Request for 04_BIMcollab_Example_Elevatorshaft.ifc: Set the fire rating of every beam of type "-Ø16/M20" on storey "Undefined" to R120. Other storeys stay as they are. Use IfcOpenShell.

First a look at what the model holds.

```python
import ifcopenshell
import ifcopenshell.util.element

model = ifcopenshell.open("04_BIMcollab_Example_Elevatorshaft.ifc")
print(model.schema)
storey = next(s for s in model.by_type("IfcBuildingStorey") if s.Name == "Undefined")
beams = [e for e in ifcopenshell.util.element.get_decomposition(storey) if e.is_a("IfcBeam")]
seen = {}
for e in beams:
    element_type = ifcopenshell.util.element.get_type(e)
    key = (element_type.Name if element_type != e and element_type else None, ifcopenshell.util.element.get_pset(e, "Pset_BeamCommon", "FireRating"))
    seen[key] = seen.get(key, 0) + 1
for (name, value), count in sorted(seen.items(), key=str):
    print(count, "x", name, "|", value)
```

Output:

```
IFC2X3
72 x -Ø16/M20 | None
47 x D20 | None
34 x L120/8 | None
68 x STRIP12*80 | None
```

```python
import ifcopenshell
import ifcopenshell.api.pset
import ifcopenshell.util.element

model = ifcopenshell.open("04_BIMcollab_Example_Elevatorshaft.ifc")

storey = next(s for s in model.by_type("IfcBuildingStorey") if s.Name == "Undefined")
beams = [e for e in ifcopenshell.util.element.get_decomposition(storey) if e.is_a("IfcBeam")]

count = 0
for e in beams:
    element_type = ifcopenshell.util.element.get_type(e)
    if element_type in (None, e) or element_type.Name != "-Ø16/M20":
        continue
    # add_pset returns the element's existing set when there is one.
    pset = ifcopenshell.api.pset.add_pset(model, product=e, name="Pset_BeamCommon")
    ifcopenshell.api.pset.edit_pset(model, pset=pset, properties={"FireRating": "R120"})
    count += 1

print(count, "beams updated")

model.write("04_BIMcollab_Example_Elevatorshaft-out.ifc")
```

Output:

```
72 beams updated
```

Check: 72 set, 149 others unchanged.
